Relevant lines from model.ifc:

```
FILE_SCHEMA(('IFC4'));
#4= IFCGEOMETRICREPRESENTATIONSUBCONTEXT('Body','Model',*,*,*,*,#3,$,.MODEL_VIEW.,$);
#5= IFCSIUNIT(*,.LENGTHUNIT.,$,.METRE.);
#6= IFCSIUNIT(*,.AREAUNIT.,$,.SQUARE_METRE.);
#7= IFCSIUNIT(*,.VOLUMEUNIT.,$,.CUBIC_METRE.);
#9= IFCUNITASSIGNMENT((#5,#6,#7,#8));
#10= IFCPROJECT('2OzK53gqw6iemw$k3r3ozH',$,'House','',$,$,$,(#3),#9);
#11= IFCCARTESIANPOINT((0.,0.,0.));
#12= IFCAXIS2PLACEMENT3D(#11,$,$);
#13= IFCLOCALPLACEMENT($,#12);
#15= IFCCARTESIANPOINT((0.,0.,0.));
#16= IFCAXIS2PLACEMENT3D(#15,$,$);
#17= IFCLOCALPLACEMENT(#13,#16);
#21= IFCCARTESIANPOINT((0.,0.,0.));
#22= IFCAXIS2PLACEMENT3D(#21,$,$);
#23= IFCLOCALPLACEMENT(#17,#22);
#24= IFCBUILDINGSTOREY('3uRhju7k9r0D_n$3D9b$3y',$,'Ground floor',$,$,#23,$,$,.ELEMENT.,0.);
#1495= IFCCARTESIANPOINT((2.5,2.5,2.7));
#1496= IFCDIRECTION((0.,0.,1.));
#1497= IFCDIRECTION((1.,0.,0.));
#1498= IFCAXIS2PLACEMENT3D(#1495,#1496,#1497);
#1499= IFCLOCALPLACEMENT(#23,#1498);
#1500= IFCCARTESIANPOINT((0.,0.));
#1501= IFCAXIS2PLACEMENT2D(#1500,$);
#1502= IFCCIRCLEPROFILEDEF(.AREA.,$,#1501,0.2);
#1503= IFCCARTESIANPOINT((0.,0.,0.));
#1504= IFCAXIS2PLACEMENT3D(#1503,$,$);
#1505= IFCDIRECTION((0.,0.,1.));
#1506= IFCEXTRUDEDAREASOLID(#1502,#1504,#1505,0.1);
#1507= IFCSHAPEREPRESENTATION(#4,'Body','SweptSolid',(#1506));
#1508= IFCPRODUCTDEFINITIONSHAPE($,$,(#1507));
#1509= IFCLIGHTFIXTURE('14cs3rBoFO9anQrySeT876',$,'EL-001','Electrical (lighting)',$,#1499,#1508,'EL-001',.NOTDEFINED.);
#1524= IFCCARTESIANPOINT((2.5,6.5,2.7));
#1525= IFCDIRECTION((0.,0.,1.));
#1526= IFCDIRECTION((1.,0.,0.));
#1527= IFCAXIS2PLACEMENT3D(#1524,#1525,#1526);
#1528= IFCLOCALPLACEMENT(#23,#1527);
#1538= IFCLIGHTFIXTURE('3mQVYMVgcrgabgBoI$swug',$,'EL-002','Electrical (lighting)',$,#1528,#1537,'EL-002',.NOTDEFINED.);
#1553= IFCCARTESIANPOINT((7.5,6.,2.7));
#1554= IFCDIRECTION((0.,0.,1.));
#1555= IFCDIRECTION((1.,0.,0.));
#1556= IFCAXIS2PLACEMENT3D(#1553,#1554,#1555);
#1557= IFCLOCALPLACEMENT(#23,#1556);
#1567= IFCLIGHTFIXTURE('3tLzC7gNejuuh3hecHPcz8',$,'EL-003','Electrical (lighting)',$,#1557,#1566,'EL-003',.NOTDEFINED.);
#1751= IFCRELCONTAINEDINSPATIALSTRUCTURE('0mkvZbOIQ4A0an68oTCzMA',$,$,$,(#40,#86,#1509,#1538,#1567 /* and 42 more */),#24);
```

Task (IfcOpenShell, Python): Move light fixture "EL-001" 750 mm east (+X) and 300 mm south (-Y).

```python
import ifcopenshell
import ifcopenshell.api.geometry
import ifcopenshell.util.placement
import ifcopenshell.util.unit

model = ifcopenshell.open("model.ifc")
unit_scale = ifcopenshell.util.unit.calculate_unit_scale(model)

item = model.by_guid("14cs3rBoFO9anQrySeT876")
matrix = ifcopenshell.util.placement.get_local_placement(item.ObjectPlacement)
matrix[0, 3] += 0.75 / unit_scale
matrix[1, 3] -= 0.3 / unit_scale
ifcopenshell.api.geometry.edit_object_placement(model, product=item, matrix=matrix, is_si=False)

print(ifcopenshell.util.placement.get_local_placement(item.ObjectPlacement).round(3) + 0.0)

model.write("model_v2.ifc")
```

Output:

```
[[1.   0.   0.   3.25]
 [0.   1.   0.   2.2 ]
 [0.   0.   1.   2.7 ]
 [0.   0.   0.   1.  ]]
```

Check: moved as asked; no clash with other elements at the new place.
